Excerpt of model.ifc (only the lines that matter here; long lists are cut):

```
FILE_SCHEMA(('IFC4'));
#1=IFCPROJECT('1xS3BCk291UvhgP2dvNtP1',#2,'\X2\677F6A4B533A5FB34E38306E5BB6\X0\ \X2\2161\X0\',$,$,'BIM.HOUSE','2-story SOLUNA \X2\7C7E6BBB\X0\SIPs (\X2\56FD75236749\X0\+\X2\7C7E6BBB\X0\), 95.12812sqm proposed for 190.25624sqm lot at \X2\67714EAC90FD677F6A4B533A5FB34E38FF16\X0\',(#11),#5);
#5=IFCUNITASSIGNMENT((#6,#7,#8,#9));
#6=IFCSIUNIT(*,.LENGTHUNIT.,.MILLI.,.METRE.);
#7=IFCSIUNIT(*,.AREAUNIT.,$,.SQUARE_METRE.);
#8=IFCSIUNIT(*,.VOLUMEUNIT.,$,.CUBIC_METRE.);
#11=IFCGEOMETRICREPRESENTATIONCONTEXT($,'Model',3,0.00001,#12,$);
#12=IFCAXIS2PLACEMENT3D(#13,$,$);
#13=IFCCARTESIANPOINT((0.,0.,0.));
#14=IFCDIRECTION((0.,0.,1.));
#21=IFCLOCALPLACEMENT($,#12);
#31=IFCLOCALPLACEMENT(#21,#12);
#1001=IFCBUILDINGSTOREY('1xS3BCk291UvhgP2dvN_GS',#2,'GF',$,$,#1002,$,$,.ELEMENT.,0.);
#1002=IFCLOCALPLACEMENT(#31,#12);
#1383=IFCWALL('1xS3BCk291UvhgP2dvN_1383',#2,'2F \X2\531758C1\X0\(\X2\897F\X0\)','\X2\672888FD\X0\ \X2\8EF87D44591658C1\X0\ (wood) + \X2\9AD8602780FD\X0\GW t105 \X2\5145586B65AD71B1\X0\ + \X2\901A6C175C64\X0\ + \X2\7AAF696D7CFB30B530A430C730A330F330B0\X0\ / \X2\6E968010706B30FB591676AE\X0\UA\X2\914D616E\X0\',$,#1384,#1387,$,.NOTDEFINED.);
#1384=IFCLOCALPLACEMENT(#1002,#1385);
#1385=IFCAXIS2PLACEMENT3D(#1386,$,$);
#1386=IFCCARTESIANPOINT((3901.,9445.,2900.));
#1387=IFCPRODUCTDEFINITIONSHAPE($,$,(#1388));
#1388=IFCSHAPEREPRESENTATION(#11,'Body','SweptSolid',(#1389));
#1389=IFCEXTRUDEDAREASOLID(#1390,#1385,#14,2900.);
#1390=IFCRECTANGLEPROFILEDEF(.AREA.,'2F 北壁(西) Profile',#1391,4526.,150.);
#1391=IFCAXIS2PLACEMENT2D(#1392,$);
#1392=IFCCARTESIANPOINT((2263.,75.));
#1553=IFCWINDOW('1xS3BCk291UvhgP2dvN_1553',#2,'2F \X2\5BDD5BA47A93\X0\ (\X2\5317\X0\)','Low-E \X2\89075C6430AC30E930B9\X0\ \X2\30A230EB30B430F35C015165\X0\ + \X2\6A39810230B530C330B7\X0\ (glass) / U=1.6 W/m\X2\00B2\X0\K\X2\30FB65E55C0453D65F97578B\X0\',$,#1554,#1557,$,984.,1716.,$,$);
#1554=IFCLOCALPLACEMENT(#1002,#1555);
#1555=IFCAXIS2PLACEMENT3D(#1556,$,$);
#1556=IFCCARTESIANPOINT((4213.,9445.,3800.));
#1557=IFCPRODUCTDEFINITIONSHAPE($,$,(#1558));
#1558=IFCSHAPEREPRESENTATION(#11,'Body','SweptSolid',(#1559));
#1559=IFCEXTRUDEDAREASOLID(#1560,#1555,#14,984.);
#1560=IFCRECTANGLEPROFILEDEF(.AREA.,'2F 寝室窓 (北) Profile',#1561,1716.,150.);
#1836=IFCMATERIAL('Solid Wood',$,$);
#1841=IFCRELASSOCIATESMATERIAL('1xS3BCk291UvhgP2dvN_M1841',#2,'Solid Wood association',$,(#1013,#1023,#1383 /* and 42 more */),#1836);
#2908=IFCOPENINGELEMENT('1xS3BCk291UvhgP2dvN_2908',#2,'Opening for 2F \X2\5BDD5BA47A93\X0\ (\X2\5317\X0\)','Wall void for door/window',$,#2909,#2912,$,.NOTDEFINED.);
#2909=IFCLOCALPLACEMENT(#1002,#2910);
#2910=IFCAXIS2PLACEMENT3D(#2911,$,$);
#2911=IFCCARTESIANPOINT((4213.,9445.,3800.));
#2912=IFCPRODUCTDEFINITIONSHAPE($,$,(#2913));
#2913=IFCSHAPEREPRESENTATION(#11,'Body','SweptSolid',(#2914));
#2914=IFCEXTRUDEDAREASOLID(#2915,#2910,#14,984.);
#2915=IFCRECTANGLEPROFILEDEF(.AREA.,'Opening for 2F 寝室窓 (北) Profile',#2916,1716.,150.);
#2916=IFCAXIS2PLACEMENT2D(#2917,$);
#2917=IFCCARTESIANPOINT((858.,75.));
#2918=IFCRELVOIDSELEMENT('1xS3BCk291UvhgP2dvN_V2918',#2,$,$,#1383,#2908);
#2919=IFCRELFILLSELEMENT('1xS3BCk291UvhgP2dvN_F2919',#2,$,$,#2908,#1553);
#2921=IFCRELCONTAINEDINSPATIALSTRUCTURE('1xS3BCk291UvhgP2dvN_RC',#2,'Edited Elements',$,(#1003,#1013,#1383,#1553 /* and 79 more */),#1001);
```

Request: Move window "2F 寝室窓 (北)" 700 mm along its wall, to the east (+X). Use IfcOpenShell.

```python
import ifcopenshell
import ifcopenshell.api.geometry
import ifcopenshell.util.placement
import ifcopenshell.util.unit

model = ifcopenshell.open("model.ifc")
unit_scale = ifcopenshell.util.unit.calculate_unit_scale(model)

window = model.by_id(1553)
opening = window.FillsVoids[0].RelatingOpeningElement
wall = opening.VoidsElements[0].RelatingBuildingElement

wall_matrix = ifcopenshell.util.placement.get_local_placement(wall.ObjectPlacement)
shift = wall_matrix[:3, 0] * 0.7 / unit_scale
before = ifcopenshell.util.placement.get_local_placement(window.ObjectPlacement)[:3, 3].copy()

# The window is not placed relative to its opening, so move both.
for product in (opening, window):
    matrix = ifcopenshell.util.placement.get_local_placement(product.ObjectPlacement)
    matrix[:3, 3] += shift
    ifcopenshell.api.geometry.edit_object_placement(model, product=product, matrix=matrix, is_si=False)

after = ifcopenshell.util.placement.get_local_placement(window.ObjectPlacement)[:3, 3]
print("window moved by", (after - before).round(3) + 0.0)

model.write("model_rev.ifc")
```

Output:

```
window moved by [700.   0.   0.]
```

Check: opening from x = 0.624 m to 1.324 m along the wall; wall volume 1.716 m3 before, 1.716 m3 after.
